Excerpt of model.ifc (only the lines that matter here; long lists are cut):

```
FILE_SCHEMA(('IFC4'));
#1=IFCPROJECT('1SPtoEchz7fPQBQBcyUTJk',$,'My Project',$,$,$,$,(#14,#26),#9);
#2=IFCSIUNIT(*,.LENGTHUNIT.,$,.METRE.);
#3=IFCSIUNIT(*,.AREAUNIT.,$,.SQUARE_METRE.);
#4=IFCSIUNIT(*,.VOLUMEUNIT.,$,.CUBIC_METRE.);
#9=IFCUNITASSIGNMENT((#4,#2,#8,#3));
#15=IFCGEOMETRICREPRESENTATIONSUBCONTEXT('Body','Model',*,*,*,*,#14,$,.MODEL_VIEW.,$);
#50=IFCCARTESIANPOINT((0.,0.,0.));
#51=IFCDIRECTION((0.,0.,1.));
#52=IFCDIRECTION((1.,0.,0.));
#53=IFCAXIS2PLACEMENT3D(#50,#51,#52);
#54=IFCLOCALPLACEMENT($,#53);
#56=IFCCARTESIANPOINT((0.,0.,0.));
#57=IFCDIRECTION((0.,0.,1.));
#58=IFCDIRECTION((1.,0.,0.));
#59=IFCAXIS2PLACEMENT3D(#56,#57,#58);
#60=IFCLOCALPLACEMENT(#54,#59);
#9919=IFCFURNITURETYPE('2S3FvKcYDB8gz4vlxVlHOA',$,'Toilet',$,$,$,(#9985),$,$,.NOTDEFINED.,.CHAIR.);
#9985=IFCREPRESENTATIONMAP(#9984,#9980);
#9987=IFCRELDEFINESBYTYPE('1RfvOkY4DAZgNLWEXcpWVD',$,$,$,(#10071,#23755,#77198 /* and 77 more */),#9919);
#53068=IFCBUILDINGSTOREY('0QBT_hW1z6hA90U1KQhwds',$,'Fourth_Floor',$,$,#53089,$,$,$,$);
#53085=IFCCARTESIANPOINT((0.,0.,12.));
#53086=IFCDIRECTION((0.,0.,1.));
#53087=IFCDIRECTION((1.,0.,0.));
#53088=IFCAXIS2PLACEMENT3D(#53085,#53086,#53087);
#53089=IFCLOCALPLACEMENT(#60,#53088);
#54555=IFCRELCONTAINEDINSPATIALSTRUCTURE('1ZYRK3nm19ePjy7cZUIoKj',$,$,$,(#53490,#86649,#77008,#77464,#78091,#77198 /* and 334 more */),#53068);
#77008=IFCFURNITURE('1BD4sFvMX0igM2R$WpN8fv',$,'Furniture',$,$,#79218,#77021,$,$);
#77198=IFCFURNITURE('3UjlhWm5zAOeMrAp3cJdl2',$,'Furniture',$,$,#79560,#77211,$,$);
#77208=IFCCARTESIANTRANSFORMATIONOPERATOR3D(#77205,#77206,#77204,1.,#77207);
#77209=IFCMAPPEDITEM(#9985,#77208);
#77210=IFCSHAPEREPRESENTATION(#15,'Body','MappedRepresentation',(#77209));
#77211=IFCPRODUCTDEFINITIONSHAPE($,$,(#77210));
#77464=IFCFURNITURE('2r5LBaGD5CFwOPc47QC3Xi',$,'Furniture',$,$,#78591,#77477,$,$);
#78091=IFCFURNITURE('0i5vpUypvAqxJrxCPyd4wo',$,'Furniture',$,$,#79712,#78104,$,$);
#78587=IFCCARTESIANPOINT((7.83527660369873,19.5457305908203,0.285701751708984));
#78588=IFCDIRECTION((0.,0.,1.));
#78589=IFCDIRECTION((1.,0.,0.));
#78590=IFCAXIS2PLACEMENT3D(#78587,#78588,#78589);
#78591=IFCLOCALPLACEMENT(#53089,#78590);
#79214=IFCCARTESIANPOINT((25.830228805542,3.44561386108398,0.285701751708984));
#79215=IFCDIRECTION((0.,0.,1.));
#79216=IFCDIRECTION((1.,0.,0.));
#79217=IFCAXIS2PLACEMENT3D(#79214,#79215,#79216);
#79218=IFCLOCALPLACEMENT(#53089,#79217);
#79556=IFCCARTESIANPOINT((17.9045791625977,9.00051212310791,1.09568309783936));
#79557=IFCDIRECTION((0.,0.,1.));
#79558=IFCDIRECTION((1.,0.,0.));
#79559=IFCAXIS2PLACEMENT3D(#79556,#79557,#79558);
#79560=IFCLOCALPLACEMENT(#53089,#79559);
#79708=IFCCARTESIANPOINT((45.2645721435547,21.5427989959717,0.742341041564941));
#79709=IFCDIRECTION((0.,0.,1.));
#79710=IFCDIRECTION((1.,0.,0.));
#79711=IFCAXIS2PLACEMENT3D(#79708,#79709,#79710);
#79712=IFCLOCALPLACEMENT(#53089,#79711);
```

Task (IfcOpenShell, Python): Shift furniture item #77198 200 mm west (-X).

```python
import ifcopenshell
import ifcopenshell.api.geometry
import ifcopenshell.util.placement

model = ifcopenshell.open("model.ifc")

item = model.by_guid("3UjlhWm5zAOeMrAp3cJdl2")
matrix = ifcopenshell.util.placement.get_local_placement(item.ObjectPlacement)
matrix[0, 3] -= 0.2
ifcopenshell.api.geometry.edit_object_placement(model, product=item, matrix=matrix, is_si=False)

print(ifcopenshell.util.placement.get_local_placement(item.ObjectPlacement).round(3) + 0.0)

model.write("model_v2.ifc")
```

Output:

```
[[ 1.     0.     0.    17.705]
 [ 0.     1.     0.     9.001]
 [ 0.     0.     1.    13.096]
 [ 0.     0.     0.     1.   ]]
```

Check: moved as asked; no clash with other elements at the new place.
